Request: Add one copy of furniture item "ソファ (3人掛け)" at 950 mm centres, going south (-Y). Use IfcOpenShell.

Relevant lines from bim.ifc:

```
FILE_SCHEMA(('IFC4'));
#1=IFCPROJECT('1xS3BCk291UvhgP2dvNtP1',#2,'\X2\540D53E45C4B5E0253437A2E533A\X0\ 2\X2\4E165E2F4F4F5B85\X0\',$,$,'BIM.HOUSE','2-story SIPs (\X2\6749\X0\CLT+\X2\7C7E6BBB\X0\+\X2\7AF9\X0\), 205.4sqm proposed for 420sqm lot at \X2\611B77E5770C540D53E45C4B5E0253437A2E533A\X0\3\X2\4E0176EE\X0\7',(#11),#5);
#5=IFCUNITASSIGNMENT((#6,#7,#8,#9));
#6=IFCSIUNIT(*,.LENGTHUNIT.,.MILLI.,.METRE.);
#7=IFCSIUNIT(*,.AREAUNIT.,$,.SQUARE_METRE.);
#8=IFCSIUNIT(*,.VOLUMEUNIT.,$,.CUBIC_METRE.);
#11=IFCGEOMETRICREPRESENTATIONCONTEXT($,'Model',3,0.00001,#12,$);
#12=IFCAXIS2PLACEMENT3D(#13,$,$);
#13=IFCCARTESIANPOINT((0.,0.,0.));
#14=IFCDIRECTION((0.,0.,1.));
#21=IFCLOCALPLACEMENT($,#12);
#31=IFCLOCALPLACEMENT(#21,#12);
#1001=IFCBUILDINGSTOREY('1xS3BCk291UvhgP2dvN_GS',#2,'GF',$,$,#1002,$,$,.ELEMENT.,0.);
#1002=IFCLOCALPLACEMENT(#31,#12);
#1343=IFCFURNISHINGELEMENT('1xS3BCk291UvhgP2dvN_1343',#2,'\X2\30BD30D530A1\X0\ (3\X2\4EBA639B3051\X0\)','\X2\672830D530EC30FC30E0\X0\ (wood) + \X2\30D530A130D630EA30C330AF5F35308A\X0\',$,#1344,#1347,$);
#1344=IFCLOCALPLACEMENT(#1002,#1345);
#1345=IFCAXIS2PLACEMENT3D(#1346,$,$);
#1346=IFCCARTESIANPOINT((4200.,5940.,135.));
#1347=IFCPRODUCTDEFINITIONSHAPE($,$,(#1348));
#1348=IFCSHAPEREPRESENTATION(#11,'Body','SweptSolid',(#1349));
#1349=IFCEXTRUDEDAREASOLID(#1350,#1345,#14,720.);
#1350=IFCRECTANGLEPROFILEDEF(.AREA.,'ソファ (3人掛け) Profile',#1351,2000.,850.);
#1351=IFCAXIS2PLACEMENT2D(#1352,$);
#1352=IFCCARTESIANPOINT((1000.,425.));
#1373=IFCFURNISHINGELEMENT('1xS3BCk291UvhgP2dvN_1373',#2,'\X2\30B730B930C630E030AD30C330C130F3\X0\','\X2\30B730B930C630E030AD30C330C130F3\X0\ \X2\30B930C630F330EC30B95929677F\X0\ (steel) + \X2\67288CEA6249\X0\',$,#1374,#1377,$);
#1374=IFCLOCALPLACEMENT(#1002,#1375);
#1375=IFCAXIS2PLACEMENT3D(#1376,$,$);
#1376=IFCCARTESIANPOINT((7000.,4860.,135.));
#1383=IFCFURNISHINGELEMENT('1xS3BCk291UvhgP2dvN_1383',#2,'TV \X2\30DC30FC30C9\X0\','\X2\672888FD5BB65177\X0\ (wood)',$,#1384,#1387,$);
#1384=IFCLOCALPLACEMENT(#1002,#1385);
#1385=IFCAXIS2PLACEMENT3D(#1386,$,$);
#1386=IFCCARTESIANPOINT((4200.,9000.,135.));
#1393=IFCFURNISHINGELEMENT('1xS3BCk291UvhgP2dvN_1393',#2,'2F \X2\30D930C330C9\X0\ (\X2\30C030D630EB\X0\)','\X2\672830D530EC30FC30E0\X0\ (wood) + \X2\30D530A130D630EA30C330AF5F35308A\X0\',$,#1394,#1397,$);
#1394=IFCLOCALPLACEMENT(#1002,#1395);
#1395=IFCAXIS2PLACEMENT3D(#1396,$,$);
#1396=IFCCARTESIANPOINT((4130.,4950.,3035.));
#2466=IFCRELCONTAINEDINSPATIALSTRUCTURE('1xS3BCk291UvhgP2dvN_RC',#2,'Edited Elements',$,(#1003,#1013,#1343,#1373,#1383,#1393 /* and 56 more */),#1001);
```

```python
import numpy as np
import ifcopenshell
import ifcopenshell.api.geometry
import ifcopenshell.api.root
import ifcopenshell.util.element
import ifcopenshell.util.placement
import ifcopenshell.util.unit

model = ifcopenshell.open("bim.ifc")
unit_scale = ifcopenshell.util.unit.calculate_unit_scale(model)


def reuse_history(source, copy):
    """copy_class also copies each property set's owner history, people and application; keep the originals."""
    for rel in copy.IsDefinedBy:
        if rel.is_a("IfcRelDefinesByProperties") and (history := rel.RelatingPropertyDefinition.OwnerHistory):
            rel.RelatingPropertyDefinition.OwnerHistory = source.OwnerHistory
            ifcopenshell.util.element.remove_deep2(model, history)


source = model.by_id(1343)
base = ifcopenshell.util.placement.get_local_placement(source.ObjectPlacement)
step = np.array([0.0, -1.0, 0.0]) * 0.95 / unit_scale

for i in range(1, 2):
    copy = ifcopenshell.api.root.copy_class(model, product=source)
    copy.Representation = ifcopenshell.util.element.copy_deep(
        model, source.Representation, exclude=["IfcGeometricRepresentationContext", "IfcRepresentationMap"]
    )
    reuse_history(source, copy)
    matrix = base.copy()
    matrix[:3, 3] += i * step
    print("added at", matrix[:3, 3].round(3) + 0.0)
    ifcopenshell.api.geometry.edit_object_placement(model, product=copy, matrix=matrix, is_si=False)

model.write("bim_v2.ifc")
```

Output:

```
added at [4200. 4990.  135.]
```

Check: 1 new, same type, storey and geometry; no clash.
